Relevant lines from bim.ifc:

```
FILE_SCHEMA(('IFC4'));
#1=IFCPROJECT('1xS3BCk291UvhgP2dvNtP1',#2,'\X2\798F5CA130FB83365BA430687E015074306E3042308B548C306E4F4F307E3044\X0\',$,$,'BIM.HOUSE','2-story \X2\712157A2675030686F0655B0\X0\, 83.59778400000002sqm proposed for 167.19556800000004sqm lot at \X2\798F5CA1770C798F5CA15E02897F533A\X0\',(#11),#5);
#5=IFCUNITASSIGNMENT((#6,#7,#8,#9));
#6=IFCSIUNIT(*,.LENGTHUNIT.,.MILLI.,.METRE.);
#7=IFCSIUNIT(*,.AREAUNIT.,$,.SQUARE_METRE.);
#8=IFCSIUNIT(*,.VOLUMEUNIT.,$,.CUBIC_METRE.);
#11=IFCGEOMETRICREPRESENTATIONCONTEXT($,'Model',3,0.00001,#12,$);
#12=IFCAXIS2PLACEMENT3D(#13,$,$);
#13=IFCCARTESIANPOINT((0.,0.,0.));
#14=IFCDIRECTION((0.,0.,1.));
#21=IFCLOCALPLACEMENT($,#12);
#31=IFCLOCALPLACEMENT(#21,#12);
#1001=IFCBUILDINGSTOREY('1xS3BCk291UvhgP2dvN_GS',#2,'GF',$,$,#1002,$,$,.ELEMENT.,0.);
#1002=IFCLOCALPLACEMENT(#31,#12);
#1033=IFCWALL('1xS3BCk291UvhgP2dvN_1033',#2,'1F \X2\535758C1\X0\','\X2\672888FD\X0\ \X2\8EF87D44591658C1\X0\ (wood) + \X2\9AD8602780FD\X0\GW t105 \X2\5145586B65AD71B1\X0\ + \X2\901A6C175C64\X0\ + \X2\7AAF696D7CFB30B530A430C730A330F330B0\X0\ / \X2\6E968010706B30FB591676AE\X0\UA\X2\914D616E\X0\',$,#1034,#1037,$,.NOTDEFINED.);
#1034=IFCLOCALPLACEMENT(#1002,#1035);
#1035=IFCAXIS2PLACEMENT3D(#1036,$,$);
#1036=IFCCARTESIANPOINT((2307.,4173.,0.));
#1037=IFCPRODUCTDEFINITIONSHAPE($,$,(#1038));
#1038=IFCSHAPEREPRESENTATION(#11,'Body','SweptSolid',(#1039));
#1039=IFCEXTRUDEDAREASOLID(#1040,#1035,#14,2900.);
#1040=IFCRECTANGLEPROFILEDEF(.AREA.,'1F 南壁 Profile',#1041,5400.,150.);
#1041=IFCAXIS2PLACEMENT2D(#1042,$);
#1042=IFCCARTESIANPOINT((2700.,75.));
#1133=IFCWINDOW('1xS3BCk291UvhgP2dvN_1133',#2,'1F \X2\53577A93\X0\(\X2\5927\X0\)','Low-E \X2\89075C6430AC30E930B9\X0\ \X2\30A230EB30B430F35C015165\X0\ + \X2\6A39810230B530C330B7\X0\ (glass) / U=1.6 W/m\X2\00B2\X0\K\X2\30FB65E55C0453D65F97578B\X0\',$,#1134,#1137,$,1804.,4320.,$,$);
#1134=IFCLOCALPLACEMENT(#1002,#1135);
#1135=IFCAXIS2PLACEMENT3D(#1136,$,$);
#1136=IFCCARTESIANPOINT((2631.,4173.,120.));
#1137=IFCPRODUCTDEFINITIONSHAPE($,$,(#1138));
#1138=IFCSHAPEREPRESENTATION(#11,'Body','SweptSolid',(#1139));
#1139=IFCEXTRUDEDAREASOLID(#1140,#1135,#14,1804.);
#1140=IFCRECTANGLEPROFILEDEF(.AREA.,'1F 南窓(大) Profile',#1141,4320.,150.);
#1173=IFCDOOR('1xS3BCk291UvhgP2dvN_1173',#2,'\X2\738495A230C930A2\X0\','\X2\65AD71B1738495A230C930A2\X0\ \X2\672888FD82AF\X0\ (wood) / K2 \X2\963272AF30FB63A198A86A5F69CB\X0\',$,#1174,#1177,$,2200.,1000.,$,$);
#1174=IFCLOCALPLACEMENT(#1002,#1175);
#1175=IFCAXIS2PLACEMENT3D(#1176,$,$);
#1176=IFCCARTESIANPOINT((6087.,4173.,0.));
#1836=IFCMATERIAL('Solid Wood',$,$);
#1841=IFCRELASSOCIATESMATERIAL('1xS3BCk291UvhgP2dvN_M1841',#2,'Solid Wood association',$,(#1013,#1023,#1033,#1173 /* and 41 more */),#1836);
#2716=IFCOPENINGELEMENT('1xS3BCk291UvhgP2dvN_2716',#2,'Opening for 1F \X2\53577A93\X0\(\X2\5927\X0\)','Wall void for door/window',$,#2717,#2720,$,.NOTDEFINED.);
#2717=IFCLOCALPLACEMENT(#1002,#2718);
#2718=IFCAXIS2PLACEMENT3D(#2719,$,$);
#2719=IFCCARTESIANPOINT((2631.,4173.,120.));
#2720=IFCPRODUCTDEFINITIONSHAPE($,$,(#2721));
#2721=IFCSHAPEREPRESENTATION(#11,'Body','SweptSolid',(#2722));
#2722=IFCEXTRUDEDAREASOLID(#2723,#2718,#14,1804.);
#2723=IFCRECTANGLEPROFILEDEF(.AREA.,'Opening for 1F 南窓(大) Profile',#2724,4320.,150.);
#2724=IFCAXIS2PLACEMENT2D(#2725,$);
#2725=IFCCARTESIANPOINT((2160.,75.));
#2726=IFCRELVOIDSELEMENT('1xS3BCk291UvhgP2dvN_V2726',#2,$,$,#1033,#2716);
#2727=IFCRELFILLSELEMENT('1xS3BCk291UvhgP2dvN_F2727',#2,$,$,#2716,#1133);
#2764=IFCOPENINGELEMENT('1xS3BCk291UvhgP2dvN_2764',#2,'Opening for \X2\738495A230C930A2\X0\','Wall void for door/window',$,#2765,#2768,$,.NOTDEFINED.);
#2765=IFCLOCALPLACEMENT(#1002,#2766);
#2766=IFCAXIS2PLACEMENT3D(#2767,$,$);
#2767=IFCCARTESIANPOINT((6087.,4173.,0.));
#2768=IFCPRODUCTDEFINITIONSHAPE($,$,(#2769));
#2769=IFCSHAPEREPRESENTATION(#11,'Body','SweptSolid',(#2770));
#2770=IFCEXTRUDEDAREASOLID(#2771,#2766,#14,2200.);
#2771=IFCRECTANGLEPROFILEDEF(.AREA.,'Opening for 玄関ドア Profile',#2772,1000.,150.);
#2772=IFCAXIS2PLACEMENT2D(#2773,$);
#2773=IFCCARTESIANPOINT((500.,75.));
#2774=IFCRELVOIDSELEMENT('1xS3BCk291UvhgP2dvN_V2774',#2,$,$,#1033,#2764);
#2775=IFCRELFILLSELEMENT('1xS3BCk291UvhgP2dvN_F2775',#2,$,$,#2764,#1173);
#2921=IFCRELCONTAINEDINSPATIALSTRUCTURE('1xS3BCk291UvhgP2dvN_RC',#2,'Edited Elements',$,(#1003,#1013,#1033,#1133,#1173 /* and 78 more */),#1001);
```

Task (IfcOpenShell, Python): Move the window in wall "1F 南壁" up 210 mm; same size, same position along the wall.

```python
import numpy as np
import ifcopenshell
import ifcopenshell.api.geometry
import ifcopenshell.util.placement
import ifcopenshell.util.unit

model = ifcopenshell.open("bim.ifc")
unit_scale = ifcopenshell.util.unit.calculate_unit_scale(model)

window = model.by_id(1133)
opening = window.FillsVoids[0].RelatingOpeningElement
dz = 210.0

shift = np.array([0.0, 0.0, dz])
# The window is not placed relative to its opening, so move both.
for product in (opening, window):
    matrix = ifcopenshell.util.placement.get_local_placement(product.ObjectPlacement)
    matrix[:3, 3] += shift
    ifcopenshell.api.geometry.edit_object_placement(model, product=product, matrix=matrix, is_si=False)

print(f"moved by {dz * unit_scale:+.3f} m")

model.write("bim_rev.ifc")
```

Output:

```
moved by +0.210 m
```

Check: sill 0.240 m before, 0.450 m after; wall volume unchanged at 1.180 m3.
